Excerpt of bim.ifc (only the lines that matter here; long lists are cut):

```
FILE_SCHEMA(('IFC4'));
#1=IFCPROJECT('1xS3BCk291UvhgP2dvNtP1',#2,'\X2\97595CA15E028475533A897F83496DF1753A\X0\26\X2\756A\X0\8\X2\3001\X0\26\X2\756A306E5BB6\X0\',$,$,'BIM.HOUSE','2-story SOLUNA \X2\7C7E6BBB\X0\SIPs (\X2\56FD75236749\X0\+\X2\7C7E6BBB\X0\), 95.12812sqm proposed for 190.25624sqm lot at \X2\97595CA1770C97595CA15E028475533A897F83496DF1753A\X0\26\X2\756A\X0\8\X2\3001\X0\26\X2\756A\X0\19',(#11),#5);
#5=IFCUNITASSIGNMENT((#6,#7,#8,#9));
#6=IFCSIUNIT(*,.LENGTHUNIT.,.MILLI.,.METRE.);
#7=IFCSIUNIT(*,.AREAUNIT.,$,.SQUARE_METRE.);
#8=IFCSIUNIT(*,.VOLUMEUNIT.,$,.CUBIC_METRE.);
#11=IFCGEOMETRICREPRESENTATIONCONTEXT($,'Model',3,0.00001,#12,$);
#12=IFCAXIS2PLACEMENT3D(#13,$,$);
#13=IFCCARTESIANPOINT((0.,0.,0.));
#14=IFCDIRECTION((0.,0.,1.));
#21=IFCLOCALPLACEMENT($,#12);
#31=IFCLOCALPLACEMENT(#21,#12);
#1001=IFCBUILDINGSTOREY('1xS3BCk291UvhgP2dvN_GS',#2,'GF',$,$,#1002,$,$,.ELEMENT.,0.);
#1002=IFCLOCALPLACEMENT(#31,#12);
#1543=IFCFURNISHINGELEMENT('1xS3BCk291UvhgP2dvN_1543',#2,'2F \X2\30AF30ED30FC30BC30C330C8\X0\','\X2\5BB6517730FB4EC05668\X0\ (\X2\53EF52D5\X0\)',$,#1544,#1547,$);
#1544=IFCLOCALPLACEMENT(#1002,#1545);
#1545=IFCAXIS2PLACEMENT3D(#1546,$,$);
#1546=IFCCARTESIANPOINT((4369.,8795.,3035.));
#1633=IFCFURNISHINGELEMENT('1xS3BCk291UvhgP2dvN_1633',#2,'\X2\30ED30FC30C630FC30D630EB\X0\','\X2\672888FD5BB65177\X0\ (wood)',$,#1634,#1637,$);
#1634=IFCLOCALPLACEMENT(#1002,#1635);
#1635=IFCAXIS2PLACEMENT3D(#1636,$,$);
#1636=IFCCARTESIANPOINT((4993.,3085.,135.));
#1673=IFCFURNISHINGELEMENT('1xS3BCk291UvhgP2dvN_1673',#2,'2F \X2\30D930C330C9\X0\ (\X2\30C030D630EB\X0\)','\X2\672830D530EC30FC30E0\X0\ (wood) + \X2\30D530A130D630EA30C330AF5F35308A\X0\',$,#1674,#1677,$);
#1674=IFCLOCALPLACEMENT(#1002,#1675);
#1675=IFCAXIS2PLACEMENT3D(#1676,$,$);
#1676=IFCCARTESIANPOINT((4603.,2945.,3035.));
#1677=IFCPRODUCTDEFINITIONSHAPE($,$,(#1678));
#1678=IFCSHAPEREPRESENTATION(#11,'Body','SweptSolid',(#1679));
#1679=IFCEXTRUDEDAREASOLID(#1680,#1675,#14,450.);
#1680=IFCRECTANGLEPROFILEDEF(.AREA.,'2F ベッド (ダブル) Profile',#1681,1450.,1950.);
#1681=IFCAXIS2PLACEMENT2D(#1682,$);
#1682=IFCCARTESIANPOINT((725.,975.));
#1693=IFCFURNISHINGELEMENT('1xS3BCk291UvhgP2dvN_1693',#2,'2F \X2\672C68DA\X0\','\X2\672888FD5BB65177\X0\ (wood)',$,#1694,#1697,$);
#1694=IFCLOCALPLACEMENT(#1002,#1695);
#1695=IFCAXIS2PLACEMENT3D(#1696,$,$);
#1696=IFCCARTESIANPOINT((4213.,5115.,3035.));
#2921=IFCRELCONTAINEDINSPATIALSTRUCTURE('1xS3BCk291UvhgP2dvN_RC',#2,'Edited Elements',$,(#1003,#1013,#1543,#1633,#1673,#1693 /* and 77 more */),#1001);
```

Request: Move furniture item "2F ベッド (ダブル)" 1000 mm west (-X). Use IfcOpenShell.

```python
import ifcopenshell
import ifcopenshell.api.geometry
import ifcopenshell.util.placement

model = ifcopenshell.open("bim.ifc")

item = model.by_guid("1xS3BCk291UvhgP2dvN_1673")
matrix = ifcopenshell.util.placement.get_local_placement(item.ObjectPlacement)
matrix[0, 3] -= 1000.0
ifcopenshell.api.geometry.edit_object_placement(model, product=item, matrix=matrix, is_si=False)

print(ifcopenshell.util.placement.get_local_placement(item.ObjectPlacement).round(3) + 0.0)

model.write("bim_rev.ifc")
```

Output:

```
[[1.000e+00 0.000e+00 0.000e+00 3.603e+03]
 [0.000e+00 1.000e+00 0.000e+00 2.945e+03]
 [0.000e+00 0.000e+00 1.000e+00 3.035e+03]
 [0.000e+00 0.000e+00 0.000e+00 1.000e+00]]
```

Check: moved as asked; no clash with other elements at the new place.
